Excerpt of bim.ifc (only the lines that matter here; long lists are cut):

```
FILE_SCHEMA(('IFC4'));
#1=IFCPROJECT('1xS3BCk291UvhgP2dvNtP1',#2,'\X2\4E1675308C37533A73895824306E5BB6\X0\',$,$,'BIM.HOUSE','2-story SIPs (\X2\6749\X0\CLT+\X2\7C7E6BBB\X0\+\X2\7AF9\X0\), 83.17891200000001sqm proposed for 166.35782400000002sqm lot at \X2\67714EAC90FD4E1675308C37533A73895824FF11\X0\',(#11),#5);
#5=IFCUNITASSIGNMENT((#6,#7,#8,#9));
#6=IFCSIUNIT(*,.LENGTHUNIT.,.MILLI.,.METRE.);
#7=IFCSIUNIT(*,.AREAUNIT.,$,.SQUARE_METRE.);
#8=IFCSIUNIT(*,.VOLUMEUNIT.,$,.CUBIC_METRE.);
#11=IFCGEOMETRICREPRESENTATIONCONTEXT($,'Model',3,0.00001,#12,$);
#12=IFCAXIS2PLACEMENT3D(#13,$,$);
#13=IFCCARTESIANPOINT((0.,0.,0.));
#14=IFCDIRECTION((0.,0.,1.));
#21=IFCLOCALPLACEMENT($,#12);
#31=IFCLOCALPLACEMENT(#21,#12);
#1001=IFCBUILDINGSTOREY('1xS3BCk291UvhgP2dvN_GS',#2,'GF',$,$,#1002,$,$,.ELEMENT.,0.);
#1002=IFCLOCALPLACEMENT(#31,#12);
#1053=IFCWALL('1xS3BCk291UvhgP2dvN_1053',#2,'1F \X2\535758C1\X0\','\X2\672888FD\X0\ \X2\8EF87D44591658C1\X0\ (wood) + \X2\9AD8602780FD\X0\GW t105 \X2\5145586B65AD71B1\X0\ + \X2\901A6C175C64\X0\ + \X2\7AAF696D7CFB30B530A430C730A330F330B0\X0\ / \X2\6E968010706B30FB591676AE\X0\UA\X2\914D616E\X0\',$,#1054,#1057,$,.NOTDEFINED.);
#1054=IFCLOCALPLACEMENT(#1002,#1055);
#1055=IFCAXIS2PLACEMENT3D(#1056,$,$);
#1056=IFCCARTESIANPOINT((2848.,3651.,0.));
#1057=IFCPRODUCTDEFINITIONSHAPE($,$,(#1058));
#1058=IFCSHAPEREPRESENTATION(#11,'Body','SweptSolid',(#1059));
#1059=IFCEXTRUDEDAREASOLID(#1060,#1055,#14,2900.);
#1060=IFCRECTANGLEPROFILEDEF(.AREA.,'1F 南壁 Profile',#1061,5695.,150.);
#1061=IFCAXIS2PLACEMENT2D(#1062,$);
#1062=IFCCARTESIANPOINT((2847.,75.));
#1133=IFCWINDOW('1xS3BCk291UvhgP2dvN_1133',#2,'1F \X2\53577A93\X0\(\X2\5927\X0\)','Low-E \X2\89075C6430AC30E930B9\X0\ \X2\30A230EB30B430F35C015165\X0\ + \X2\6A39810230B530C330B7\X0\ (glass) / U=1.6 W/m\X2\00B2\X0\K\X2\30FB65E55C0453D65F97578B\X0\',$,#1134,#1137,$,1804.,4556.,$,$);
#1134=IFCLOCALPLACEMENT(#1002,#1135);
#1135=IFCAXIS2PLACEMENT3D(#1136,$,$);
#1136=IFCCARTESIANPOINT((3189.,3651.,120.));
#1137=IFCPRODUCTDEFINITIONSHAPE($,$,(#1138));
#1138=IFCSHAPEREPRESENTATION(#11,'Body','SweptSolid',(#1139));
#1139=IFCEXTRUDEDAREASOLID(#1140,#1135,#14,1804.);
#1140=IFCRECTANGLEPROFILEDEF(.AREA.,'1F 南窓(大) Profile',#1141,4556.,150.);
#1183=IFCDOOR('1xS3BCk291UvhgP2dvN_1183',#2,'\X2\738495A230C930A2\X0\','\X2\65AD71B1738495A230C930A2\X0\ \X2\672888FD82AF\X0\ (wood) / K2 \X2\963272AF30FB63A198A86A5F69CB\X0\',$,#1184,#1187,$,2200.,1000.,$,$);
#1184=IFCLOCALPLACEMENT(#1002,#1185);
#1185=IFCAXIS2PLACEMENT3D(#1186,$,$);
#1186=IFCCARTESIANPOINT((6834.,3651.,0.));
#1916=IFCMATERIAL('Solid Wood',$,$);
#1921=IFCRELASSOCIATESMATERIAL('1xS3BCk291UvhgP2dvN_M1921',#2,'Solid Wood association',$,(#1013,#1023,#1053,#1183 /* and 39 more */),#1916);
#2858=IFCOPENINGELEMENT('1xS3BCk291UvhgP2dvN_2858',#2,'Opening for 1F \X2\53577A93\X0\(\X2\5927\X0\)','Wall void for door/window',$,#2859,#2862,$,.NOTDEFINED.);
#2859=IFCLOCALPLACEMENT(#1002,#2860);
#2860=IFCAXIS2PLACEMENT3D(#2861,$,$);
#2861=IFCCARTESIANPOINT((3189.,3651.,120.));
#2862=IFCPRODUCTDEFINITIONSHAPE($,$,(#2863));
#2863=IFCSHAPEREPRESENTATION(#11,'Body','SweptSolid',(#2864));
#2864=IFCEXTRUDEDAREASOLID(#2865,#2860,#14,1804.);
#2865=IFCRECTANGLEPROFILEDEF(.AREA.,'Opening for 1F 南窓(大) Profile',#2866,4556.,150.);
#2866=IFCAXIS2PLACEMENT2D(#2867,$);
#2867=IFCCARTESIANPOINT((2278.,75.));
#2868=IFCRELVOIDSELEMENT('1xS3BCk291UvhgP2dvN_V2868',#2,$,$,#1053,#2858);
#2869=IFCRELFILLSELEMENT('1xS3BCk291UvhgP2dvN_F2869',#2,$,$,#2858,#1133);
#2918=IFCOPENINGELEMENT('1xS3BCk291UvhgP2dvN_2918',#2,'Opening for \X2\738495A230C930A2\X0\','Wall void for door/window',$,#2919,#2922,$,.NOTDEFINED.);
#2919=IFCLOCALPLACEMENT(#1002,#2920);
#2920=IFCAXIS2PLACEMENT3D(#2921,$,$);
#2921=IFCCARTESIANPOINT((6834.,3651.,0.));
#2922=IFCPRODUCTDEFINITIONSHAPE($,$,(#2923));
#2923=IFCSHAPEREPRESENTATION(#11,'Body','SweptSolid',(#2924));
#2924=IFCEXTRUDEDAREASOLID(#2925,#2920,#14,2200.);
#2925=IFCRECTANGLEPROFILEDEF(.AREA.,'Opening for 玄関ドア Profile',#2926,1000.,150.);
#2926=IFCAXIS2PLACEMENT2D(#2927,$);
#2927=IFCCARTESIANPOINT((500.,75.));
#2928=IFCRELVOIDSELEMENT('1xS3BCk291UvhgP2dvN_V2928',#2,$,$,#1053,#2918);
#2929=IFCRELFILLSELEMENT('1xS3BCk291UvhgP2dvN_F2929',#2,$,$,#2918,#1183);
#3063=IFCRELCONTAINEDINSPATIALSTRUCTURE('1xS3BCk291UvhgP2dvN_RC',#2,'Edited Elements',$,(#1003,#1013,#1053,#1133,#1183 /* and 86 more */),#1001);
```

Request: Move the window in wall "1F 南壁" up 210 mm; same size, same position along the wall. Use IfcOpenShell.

```python
import numpy as np
import ifcopenshell
import ifcopenshell.api.geometry
import ifcopenshell.util.placement
import ifcopenshell.util.unit

model = ifcopenshell.open("bim.ifc")
unit_scale = ifcopenshell.util.unit.calculate_unit_scale(model)

window = model.by_id(1133)
opening = window.FillsVoids[0].RelatingOpeningElement
dz = 0.21 / unit_scale

shift = np.array([0.0, 0.0, dz])
# The window is not placed relative to its opening, so move both.
for product in (opening, window):
    matrix = ifcopenshell.util.placement.get_local_placement(product.ObjectPlacement)
    matrix[:3, 3] += shift
    ifcopenshell.api.geometry.edit_object_placement(model, product=product, matrix=matrix, is_si=False)

print(f"moved by {dz * unit_scale:+.3f} m")

model.write("bim_v2.ifc")
```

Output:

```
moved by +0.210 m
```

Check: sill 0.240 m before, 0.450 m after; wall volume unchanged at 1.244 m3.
